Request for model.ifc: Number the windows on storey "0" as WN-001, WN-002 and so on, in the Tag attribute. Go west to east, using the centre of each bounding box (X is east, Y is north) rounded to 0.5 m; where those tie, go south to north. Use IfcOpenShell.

First a look at what the model holds.

```python
import ifcopenshell
import ifcopenshell.util.element
import ifcopenshell.util.placement

model = ifcopenshell.open("model.ifc")
print(model.schema)
storey = next(s for s in model.by_type("IfcBuildingStorey") if s.Name == "0")
windows = [e for e in ifcopenshell.util.element.get_decomposition(storey) if e.is_a("IfcWindow")]
for e in sorted(windows, key=lambda e: e.id()):
    origin = ifcopenshell.util.placement.get_local_placement(e.ObjectPlacement)[:3, 3]
    print(e.id(), e.Tag, e.Name, origin.round(2) + 0.0, sep=" | ")
```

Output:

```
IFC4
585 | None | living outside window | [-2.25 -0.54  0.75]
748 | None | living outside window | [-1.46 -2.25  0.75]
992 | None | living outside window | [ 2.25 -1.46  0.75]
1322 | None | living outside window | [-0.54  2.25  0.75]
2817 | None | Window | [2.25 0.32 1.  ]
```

```python
import ifcopenshell
import ifcopenshell.geom
import ifcopenshell.util.element
import ifcopenshell.util.shape

model = ifcopenshell.open("model.ifc")
settings = ifcopenshell.geom.settings()
settings.set("use-world-coords", True)


def centre(element):
    shape = ifcopenshell.geom.create_shape(settings, element)
    return ifcopenshell.util.shape.get_bbox_centroid(shape.geometry)


storey = next(s for s in model.by_type("IfcBuildingStorey") if s.Name == "0")
windows = [e for e in ifcopenshell.util.element.get_decomposition(storey) if e.is_a("IfcWindow")]

# Insertion points can sit at a corner or the storey origin, so sort by the geometry (in metres).
centres = {e: centre(e) for e in windows}
windows.sort(key=lambda e: (round(centres[e][0] / 0.5), centres[e][1]))

for i, e in enumerate(windows, start=1):
    number = f"WN-0{i:02d}"
    e.Tag = number
    print(e.id(), number)

model.write("model_updated.ifc")
```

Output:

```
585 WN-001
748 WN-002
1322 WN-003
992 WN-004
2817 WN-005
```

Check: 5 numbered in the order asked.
